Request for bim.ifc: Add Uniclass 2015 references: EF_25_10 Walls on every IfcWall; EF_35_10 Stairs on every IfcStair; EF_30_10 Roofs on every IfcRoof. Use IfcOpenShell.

First a look at what the model holds.

```python
import ifcopenshell

model = ifcopenshell.open("bim.ifc")
print(model.schema)
print("classifications:", [c.Name for c in model.by_type("IfcClassification")])
for ifc_class in ("IfcDoor", "IfcRoof", "IfcStair", "IfcWall", "IfcWindow"):
    print(ifc_class, len(model.by_type(ifc_class)))
```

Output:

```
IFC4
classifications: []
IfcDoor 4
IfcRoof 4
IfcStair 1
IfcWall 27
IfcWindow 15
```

```python
import ifcopenshell
import ifcopenshell.api.classification

model = ifcopenshell.open("bim.ifc")

system = ifcopenshell.api.classification.add_classification(model, classification="Uniclass 2015")

codes = {
    "IfcWall": ("EF_25_10", "Walls"),
    "IfcStair": ("EF_35_10", "Stairs"),
    "IfcRoof": ("EF_30_10", "Roofs"),
}
for ifc_class, (code, name) in codes.items():
    products = model.by_type(ifc_class)
    ifcopenshell.api.classification.add_reference(
        model, products=products, classification=system, identification=code, name=name
    )
    print(code, len(products))

model.write("bim_rev.ifc")
```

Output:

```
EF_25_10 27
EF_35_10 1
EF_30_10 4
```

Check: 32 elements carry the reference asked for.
